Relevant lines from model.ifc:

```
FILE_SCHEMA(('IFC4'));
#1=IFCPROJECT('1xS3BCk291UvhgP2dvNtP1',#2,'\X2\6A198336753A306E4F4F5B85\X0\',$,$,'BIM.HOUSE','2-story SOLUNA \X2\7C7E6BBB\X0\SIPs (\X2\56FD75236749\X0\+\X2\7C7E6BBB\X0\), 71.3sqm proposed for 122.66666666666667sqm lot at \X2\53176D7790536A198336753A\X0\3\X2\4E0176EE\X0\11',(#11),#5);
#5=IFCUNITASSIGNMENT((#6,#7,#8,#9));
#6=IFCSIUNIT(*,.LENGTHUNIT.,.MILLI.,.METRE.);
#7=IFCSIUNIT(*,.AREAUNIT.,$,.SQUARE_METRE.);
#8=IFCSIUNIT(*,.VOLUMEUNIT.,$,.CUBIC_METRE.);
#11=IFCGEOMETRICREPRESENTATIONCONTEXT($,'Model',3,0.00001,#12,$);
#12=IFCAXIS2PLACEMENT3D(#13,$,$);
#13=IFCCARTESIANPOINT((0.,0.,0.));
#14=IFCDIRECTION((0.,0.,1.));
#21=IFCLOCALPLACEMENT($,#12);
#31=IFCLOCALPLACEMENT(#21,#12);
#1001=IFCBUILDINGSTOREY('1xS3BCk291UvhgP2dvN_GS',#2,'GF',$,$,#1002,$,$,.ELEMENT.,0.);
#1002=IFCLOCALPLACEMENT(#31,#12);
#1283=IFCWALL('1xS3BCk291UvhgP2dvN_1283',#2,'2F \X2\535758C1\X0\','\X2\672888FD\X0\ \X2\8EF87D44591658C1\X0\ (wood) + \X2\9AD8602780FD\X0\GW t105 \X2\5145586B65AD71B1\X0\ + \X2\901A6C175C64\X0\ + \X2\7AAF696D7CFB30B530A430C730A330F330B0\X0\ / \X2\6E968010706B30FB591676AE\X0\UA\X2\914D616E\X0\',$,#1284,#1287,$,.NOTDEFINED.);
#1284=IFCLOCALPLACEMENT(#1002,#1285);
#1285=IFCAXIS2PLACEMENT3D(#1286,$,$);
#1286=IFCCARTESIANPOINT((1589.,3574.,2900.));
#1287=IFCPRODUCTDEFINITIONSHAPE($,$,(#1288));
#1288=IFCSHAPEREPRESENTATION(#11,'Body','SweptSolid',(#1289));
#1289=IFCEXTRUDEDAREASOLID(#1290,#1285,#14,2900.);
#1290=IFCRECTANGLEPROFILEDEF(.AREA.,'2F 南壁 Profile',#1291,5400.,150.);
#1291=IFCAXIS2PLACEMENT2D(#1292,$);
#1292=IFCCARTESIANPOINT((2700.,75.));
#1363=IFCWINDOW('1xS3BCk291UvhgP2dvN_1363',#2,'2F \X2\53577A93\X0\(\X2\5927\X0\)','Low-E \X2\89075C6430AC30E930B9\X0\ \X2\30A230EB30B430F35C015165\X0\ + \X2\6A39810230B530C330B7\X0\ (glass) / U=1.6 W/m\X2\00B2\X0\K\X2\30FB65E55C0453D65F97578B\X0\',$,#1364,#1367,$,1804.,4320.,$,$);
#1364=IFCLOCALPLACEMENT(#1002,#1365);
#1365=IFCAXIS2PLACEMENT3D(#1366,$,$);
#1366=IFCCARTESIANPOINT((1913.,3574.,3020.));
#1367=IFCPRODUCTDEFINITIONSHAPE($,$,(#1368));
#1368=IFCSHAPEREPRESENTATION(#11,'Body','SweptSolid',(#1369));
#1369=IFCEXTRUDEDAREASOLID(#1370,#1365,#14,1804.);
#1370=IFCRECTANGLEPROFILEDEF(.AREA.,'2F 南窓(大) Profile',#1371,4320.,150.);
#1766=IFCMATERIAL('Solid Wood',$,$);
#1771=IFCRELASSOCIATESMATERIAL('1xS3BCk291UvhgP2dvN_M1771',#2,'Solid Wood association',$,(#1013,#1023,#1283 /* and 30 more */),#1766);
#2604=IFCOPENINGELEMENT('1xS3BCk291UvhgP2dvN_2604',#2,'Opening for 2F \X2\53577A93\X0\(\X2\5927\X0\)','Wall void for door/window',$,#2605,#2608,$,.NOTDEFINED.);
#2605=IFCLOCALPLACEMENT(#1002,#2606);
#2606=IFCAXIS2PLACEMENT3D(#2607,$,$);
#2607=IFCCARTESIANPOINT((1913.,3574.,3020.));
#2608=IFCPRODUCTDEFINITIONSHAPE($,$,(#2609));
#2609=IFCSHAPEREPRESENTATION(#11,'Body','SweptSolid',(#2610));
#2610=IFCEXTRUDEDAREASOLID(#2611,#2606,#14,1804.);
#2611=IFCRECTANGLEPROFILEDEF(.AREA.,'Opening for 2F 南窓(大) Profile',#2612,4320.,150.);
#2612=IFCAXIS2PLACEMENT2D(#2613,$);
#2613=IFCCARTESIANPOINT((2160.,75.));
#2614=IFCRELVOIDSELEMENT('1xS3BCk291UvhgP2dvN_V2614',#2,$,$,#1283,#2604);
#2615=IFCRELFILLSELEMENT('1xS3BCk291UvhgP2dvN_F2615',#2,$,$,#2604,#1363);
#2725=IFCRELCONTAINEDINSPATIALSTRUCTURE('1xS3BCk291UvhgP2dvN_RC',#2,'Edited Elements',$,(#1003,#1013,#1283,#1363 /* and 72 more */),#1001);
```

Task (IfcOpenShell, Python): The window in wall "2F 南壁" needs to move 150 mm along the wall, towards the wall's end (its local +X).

```python
import ifcopenshell
import ifcopenshell.api.geometry
import ifcopenshell.util.placement
import ifcopenshell.util.unit

model = ifcopenshell.open("model.ifc")
unit_scale = ifcopenshell.util.unit.calculate_unit_scale(model)

window = model.by_id(1363)
opening = window.FillsVoids[0].RelatingOpeningElement
wall = opening.VoidsElements[0].RelatingBuildingElement

wall_matrix = ifcopenshell.util.placement.get_local_placement(wall.ObjectPlacement)
shift = wall_matrix[:3, 0] * 0.15 / unit_scale
before = ifcopenshell.util.placement.get_local_placement(window.ObjectPlacement)[:3, 3].copy()

# The window is not placed relative to its opening, so move both.
for product in (opening, window):
    matrix = ifcopenshell.util.placement.get_local_placement(product.ObjectPlacement)
    matrix[:3, 3] += shift
    ifcopenshell.api.geometry.edit_object_placement(model, product=product, matrix=matrix, is_si=False)

after = ifcopenshell.util.placement.get_local_placement(window.ObjectPlacement)[:3, 3]
print("window moved by", (after - before).round(3) + 0.0)

model.write("model-out.ifc")
```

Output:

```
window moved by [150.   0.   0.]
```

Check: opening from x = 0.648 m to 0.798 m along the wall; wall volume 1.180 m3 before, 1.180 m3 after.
